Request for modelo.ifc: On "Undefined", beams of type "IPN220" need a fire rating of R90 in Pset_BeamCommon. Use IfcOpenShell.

First a look at what the model holds.

```python
import ifcopenshell
import ifcopenshell.util.element

model = ifcopenshell.open("modelo.ifc")
print(model.schema)
storey = next(s for s in model.by_type("IfcBuildingStorey") if s.Name == "Undefined")
beams = [e for e in ifcopenshell.util.element.get_decomposition(storey) if e.is_a("IfcBeam")]
seen = {}
for e in beams:
    element_type = ifcopenshell.util.element.get_type(e)
    key = (element_type.Name if element_type != e and element_type else None, ifcopenshell.util.element.get_pset(e, "Pset_BeamCommon", "FireRating"))
    seen[key] = seen.get(key, 0) + 1
for (name, value), count in sorted(seen.items(), key=str):
    print(count, "x", name, "|", value)
```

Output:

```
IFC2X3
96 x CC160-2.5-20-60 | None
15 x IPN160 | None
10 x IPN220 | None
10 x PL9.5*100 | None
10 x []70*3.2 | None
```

```python
import ifcopenshell
import ifcopenshell.api.pset
import ifcopenshell.util.element

model = ifcopenshell.open("modelo.ifc")

storey = next(s for s in model.by_type("IfcBuildingStorey") if s.Name == "Undefined")
beams = [e for e in ifcopenshell.util.element.get_decomposition(storey) if e.is_a("IfcBeam")]

count = 0
for e in beams:
    element_type = ifcopenshell.util.element.get_type(e)
    if element_type in (None, e) or element_type.Name != "IPN220":
        continue
    found = ifcopenshell.util.element.get_pset(e, "Pset_BeamCommon", should_inherit=False)
    if found:
        pset = model.by_id(found["id"])
        if len(ifcopenshell.util.element.get_elements_by_pset(pset)) > 1:
            pset = ifcopenshell.api.pset.unshare_pset(model, products=[e], pset=pset)[0]
    else:
        pset = ifcopenshell.api.pset.add_pset(model, product=e, name="Pset_BeamCommon")
    ifcopenshell.api.pset.edit_pset(model, pset=pset, properties={"FireRating": "R90"})
    count += 1

print(count, "beams updated")

model.write("modelo_updated.ifc")
```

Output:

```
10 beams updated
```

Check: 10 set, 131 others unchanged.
